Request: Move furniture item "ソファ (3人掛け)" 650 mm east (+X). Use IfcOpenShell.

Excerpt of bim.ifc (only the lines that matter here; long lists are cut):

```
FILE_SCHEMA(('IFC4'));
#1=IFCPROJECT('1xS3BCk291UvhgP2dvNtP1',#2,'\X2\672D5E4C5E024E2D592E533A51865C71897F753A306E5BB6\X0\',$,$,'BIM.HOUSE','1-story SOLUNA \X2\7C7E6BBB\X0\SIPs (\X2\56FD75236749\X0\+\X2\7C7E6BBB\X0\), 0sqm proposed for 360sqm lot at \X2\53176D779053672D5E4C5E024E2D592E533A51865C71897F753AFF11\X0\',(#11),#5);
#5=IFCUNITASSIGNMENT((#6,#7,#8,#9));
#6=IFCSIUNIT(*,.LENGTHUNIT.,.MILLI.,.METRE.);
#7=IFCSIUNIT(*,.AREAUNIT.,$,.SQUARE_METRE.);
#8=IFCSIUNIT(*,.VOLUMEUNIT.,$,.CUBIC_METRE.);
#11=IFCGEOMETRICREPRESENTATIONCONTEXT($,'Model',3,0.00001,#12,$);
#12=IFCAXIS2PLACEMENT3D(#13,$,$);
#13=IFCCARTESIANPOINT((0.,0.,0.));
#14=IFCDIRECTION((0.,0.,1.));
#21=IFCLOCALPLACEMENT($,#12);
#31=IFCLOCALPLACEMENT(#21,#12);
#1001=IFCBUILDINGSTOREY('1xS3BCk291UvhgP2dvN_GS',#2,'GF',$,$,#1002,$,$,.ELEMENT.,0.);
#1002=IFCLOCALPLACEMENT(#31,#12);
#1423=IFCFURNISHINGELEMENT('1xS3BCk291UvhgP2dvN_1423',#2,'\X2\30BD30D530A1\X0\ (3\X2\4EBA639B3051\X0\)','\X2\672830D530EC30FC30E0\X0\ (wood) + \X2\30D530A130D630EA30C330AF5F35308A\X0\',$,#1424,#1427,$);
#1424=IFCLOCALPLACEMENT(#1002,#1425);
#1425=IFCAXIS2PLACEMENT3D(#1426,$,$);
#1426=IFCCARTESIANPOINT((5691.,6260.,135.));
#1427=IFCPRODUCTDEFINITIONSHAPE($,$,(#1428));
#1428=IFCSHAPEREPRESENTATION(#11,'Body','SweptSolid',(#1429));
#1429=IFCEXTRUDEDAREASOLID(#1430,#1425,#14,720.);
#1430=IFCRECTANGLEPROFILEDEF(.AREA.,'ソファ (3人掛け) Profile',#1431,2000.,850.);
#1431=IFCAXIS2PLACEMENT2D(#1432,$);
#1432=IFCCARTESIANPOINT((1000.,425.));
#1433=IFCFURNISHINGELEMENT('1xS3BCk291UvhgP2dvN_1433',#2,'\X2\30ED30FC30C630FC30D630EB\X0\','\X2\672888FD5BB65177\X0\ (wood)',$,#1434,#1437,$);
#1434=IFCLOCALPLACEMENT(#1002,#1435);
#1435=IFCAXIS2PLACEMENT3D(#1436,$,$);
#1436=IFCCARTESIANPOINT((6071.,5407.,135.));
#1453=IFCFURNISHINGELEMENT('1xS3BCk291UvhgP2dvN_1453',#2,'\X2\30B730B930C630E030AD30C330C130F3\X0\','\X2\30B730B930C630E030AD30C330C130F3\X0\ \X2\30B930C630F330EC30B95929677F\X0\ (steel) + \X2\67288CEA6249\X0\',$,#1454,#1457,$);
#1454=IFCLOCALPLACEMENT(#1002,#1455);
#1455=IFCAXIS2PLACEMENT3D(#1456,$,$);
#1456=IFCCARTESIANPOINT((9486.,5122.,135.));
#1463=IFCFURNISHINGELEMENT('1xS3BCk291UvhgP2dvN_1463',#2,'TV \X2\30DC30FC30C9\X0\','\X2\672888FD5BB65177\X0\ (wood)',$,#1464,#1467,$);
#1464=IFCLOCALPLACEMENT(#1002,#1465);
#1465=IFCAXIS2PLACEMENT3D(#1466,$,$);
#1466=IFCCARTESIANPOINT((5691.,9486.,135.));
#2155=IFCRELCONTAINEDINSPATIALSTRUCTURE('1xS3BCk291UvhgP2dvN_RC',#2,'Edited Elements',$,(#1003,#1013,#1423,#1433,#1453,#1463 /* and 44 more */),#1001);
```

```python
import ifcopenshell
import ifcopenshell.api.geometry
import ifcopenshell.util.placement

model = ifcopenshell.open("bim.ifc")

item = model.by_guid("1xS3BCk291UvhgP2dvN_1423")
matrix = ifcopenshell.util.placement.get_local_placement(item.ObjectPlacement)
matrix[0, 3] += 650.0
ifcopenshell.api.geometry.edit_object_placement(model, product=item, matrix=matrix, is_si=False)

print(ifcopenshell.util.placement.get_local_placement(item.ObjectPlacement).round(3) + 0.0)

model.write("bim_updated.ifc")
```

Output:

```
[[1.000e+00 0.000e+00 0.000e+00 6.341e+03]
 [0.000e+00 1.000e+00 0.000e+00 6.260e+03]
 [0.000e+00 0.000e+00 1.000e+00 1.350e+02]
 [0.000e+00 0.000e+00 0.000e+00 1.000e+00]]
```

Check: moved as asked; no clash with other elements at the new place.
